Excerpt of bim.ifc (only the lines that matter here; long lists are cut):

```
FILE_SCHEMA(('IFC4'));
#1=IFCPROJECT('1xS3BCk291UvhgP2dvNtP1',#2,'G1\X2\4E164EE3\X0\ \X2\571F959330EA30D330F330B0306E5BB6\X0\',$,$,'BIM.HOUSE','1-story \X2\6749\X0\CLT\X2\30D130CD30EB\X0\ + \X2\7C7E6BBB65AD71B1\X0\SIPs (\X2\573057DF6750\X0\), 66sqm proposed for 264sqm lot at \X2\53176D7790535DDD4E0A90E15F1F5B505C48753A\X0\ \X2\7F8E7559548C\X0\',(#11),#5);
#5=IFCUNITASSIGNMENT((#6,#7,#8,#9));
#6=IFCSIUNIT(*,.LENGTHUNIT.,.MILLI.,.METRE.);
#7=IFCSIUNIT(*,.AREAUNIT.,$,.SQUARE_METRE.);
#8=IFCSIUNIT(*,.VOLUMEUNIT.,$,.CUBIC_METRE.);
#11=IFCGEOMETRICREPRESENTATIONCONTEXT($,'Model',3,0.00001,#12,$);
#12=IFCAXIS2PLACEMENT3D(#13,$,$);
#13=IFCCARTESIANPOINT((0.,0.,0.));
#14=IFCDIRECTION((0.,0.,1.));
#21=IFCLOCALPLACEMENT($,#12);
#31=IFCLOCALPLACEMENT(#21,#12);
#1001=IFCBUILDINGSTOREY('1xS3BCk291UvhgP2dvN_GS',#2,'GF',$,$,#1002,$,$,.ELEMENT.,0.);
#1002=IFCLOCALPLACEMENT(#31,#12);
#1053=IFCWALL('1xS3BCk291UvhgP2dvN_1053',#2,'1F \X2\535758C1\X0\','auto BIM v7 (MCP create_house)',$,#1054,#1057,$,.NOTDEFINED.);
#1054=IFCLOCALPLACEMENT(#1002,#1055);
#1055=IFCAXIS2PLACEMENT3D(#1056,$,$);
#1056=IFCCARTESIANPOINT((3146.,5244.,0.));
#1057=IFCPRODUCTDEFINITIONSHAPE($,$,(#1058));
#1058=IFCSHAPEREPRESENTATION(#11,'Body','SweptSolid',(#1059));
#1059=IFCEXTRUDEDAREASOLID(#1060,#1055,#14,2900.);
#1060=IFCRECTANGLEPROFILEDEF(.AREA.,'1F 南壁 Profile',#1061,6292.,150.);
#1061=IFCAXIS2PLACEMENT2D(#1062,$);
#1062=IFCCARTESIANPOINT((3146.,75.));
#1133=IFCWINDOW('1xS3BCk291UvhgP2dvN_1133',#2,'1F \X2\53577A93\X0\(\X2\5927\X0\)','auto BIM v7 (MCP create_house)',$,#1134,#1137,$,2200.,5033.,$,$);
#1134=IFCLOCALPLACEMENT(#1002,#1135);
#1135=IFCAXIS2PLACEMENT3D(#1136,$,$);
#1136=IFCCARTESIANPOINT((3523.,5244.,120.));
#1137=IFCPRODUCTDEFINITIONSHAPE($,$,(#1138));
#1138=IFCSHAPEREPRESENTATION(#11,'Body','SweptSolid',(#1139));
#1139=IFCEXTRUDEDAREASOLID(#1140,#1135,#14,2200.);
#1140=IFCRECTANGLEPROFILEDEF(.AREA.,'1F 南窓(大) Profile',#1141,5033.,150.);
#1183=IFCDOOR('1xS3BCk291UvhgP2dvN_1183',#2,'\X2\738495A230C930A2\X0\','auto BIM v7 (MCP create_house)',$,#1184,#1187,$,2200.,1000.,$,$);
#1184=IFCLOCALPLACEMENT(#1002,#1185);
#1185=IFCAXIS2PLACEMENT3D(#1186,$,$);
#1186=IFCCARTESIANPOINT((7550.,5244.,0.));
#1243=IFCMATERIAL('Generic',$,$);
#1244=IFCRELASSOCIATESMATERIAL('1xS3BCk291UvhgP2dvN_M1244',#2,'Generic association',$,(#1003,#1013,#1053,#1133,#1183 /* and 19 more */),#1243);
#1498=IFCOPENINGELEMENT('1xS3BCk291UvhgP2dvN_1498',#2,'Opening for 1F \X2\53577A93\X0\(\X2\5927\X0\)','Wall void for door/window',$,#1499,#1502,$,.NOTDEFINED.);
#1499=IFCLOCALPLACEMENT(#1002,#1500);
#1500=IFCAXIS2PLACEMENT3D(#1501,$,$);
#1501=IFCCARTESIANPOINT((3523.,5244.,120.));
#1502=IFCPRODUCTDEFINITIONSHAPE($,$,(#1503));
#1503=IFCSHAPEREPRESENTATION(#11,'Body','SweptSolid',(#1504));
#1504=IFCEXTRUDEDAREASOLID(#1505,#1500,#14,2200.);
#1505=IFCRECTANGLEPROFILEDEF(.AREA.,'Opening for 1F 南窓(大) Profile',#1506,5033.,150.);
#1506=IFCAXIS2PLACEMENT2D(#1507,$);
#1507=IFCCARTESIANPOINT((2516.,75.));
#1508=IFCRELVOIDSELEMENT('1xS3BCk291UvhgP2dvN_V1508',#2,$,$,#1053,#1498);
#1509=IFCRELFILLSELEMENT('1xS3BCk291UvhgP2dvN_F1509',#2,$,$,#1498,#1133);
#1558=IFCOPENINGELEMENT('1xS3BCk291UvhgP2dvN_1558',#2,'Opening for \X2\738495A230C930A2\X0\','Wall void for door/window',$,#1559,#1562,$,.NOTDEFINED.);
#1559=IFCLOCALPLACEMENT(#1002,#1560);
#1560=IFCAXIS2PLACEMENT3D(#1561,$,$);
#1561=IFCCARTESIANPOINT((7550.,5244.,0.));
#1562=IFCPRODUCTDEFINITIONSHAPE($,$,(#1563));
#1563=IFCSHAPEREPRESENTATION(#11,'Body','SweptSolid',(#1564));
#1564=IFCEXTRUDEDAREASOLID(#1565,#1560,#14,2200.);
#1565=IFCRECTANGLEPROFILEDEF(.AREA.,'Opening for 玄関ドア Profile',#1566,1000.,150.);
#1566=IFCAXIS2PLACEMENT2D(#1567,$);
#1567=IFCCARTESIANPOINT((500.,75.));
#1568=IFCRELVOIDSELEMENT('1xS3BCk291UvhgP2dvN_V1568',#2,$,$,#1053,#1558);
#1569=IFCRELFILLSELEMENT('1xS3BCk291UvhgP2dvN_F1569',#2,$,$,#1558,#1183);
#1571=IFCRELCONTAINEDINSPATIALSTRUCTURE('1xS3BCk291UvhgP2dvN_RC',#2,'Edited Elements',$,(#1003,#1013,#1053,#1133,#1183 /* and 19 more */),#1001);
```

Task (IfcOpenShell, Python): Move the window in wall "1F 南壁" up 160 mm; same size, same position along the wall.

```python
import numpy as np
import ifcopenshell
import ifcopenshell.api.geometry
import ifcopenshell.util.placement
import ifcopenshell.util.unit

model = ifcopenshell.open("bim.ifc")
unit_scale = ifcopenshell.util.unit.calculate_unit_scale(model)

window = model.by_guid("1xS3BCk291UvhgP2dvN_1133")
opening = window.FillsVoids[0].RelatingOpeningElement
dz = 160.0

shift = np.array([0.0, 0.0, dz])
# The window is not placed relative to its opening, so move both.
for product in (opening, window):
    matrix = ifcopenshell.util.placement.get_local_placement(product.ObjectPlacement)
    matrix[:3, 3] += shift
    ifcopenshell.api.geometry.edit_object_placement(model, product=product, matrix=matrix, is_si=False)

print(f"moved by {dz * unit_scale:+.3f} m")

model.write("bim_edited.ifc")
```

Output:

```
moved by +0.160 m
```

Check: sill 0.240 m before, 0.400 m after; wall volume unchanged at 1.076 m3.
